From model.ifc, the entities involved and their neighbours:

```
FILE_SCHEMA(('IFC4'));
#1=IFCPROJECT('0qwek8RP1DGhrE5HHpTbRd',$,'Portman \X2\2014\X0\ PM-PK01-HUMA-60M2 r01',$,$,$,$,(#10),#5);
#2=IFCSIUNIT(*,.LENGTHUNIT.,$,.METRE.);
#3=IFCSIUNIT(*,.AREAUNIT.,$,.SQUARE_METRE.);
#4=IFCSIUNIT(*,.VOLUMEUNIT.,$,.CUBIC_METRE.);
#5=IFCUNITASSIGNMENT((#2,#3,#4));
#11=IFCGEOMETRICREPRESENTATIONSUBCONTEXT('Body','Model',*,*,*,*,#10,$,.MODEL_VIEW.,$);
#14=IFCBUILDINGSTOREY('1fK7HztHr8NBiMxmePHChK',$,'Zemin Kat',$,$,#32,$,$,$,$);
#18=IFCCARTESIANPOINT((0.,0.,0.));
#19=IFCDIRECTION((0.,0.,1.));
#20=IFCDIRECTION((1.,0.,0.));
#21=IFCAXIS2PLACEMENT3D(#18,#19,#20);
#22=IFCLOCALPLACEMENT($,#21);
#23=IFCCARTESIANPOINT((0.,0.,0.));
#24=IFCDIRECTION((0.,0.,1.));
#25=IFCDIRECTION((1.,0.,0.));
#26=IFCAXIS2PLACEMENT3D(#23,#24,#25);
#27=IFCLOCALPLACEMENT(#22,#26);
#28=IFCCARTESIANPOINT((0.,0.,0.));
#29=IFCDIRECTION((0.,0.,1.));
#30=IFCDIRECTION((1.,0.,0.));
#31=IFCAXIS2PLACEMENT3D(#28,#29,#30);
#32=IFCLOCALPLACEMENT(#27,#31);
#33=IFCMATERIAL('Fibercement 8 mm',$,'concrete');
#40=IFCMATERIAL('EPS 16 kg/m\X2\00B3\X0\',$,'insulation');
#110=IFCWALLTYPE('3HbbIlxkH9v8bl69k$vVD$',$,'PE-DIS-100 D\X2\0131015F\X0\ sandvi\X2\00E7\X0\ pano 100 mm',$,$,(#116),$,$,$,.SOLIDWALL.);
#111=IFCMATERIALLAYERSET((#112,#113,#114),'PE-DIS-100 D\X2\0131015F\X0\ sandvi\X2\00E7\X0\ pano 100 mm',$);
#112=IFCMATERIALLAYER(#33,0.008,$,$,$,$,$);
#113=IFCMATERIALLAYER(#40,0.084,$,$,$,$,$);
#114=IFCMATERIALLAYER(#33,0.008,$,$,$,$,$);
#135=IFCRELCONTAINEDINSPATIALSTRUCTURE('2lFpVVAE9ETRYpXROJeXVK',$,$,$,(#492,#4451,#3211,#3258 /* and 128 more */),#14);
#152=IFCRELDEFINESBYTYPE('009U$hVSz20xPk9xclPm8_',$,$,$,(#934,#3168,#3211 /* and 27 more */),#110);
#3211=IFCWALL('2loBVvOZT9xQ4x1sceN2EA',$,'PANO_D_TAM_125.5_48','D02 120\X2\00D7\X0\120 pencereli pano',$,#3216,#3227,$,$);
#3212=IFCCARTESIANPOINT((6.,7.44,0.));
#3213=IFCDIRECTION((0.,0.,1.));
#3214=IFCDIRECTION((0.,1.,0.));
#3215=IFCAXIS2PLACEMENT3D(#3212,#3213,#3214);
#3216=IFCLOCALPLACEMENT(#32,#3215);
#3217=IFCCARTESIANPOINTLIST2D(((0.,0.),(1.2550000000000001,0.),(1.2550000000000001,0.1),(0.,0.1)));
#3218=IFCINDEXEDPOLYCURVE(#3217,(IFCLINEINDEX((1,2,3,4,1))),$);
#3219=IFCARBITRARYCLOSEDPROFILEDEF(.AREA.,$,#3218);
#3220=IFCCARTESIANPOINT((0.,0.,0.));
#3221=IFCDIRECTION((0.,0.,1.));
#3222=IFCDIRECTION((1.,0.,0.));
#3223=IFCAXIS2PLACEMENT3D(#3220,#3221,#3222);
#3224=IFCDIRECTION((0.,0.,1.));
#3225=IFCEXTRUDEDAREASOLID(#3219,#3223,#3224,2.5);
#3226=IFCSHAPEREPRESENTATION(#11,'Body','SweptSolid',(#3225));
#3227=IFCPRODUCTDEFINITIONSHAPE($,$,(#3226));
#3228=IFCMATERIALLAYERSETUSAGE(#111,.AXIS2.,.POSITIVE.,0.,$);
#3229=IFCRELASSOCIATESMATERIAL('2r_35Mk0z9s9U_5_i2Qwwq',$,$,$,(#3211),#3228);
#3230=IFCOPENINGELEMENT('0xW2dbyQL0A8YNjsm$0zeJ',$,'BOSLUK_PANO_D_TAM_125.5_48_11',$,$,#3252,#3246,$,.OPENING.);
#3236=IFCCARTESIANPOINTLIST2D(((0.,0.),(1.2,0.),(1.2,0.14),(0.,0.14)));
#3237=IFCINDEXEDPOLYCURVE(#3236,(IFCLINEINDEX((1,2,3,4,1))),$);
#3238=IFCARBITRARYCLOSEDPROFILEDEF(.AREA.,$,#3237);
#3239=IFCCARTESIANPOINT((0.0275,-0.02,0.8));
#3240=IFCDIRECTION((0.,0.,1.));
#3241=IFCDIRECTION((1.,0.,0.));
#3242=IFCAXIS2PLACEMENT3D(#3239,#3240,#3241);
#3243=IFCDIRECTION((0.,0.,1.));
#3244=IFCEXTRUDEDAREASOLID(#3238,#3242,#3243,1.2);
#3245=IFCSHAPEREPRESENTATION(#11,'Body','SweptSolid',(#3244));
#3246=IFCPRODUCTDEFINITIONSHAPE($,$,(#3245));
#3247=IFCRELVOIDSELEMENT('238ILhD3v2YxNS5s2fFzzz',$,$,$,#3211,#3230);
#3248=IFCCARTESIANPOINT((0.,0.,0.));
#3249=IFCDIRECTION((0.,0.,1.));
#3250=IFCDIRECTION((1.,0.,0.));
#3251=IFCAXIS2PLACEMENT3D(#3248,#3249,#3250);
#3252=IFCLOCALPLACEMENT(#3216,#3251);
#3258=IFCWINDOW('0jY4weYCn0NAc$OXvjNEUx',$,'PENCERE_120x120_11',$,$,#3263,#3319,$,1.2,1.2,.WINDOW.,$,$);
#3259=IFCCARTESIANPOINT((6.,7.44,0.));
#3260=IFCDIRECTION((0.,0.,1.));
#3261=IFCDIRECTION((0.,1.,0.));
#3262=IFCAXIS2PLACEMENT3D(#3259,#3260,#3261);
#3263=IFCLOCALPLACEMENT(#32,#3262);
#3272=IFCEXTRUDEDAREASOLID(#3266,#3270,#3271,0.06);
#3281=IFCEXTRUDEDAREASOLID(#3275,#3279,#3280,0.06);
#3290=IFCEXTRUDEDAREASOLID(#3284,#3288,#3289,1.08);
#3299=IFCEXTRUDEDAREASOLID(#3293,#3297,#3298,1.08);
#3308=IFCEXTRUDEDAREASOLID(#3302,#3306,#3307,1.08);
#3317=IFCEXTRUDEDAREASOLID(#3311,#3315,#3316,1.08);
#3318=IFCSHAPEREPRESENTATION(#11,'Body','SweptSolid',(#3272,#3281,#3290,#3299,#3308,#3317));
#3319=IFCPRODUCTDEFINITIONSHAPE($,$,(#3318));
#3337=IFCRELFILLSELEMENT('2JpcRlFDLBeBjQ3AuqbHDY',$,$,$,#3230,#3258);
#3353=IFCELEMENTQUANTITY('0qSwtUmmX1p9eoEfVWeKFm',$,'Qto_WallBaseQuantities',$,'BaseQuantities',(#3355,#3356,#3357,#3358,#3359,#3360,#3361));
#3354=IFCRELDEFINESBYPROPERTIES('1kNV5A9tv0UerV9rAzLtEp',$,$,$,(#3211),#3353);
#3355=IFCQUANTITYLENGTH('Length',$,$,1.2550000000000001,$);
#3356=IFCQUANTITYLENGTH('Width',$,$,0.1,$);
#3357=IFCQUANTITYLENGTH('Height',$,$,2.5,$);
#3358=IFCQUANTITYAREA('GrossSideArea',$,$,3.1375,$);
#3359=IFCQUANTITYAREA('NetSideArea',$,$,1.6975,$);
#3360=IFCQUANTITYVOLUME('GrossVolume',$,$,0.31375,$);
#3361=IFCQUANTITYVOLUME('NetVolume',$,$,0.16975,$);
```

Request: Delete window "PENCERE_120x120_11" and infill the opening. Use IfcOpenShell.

```python
import ifcopenshell
import ifcopenshell.api.feature
import ifcopenshell.api.pset
import ifcopenshell.api.root
import ifcopenshell.geom
import ifcopenshell.util.element
import ifcopenshell.util.shape
import ifcopenshell.util.unit

model = ifcopenshell.open("model.ifc")
area_scale = ifcopenshell.util.unit.calculate_unit_scale(model, "AREAUNIT")
volume_scale = ifcopenshell.util.unit.calculate_unit_scale(model, "VOLUMEUNIT")
settings = ifcopenshell.geom.settings()


def volume(element):
    """Net volume in cubic metres, openings subtracted."""
    shape = ifcopenshell.geom.create_shape(settings, element)
    return ifcopenshell.util.shape.get_volume(shape.geometry)


window = model.by_id(3258)
opening = window.FillsVoids[0].RelatingOpeningElement
wall = opening.VoidsElements[0].RelatingBuildingElement
before = volume(wall)

ifcopenshell.api.root.remove_product(model, product=window)
ifcopenshell.api.feature.remove_feature(model, feature=opening)

after = volume(wall)
thickness = 0.1  # wall thickness in metres

# Update the wall's stored quantities.
qto = model.by_id(ifcopenshell.util.element.get_pset(wall, "Qto_WallBaseQuantities", should_inherit=False)["id"])
ifcopenshell.api.pset.edit_qto(model, qto=qto, properties={
    "NetSideArea": after / thickness / area_scale,
    "NetVolume": after / volume_scale,
})

print(f"wall volume {before:.3f} -> {after:.3f} m3")

model.write("model_updated.ifc")
```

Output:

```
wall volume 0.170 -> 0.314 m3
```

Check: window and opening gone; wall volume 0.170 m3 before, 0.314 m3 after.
